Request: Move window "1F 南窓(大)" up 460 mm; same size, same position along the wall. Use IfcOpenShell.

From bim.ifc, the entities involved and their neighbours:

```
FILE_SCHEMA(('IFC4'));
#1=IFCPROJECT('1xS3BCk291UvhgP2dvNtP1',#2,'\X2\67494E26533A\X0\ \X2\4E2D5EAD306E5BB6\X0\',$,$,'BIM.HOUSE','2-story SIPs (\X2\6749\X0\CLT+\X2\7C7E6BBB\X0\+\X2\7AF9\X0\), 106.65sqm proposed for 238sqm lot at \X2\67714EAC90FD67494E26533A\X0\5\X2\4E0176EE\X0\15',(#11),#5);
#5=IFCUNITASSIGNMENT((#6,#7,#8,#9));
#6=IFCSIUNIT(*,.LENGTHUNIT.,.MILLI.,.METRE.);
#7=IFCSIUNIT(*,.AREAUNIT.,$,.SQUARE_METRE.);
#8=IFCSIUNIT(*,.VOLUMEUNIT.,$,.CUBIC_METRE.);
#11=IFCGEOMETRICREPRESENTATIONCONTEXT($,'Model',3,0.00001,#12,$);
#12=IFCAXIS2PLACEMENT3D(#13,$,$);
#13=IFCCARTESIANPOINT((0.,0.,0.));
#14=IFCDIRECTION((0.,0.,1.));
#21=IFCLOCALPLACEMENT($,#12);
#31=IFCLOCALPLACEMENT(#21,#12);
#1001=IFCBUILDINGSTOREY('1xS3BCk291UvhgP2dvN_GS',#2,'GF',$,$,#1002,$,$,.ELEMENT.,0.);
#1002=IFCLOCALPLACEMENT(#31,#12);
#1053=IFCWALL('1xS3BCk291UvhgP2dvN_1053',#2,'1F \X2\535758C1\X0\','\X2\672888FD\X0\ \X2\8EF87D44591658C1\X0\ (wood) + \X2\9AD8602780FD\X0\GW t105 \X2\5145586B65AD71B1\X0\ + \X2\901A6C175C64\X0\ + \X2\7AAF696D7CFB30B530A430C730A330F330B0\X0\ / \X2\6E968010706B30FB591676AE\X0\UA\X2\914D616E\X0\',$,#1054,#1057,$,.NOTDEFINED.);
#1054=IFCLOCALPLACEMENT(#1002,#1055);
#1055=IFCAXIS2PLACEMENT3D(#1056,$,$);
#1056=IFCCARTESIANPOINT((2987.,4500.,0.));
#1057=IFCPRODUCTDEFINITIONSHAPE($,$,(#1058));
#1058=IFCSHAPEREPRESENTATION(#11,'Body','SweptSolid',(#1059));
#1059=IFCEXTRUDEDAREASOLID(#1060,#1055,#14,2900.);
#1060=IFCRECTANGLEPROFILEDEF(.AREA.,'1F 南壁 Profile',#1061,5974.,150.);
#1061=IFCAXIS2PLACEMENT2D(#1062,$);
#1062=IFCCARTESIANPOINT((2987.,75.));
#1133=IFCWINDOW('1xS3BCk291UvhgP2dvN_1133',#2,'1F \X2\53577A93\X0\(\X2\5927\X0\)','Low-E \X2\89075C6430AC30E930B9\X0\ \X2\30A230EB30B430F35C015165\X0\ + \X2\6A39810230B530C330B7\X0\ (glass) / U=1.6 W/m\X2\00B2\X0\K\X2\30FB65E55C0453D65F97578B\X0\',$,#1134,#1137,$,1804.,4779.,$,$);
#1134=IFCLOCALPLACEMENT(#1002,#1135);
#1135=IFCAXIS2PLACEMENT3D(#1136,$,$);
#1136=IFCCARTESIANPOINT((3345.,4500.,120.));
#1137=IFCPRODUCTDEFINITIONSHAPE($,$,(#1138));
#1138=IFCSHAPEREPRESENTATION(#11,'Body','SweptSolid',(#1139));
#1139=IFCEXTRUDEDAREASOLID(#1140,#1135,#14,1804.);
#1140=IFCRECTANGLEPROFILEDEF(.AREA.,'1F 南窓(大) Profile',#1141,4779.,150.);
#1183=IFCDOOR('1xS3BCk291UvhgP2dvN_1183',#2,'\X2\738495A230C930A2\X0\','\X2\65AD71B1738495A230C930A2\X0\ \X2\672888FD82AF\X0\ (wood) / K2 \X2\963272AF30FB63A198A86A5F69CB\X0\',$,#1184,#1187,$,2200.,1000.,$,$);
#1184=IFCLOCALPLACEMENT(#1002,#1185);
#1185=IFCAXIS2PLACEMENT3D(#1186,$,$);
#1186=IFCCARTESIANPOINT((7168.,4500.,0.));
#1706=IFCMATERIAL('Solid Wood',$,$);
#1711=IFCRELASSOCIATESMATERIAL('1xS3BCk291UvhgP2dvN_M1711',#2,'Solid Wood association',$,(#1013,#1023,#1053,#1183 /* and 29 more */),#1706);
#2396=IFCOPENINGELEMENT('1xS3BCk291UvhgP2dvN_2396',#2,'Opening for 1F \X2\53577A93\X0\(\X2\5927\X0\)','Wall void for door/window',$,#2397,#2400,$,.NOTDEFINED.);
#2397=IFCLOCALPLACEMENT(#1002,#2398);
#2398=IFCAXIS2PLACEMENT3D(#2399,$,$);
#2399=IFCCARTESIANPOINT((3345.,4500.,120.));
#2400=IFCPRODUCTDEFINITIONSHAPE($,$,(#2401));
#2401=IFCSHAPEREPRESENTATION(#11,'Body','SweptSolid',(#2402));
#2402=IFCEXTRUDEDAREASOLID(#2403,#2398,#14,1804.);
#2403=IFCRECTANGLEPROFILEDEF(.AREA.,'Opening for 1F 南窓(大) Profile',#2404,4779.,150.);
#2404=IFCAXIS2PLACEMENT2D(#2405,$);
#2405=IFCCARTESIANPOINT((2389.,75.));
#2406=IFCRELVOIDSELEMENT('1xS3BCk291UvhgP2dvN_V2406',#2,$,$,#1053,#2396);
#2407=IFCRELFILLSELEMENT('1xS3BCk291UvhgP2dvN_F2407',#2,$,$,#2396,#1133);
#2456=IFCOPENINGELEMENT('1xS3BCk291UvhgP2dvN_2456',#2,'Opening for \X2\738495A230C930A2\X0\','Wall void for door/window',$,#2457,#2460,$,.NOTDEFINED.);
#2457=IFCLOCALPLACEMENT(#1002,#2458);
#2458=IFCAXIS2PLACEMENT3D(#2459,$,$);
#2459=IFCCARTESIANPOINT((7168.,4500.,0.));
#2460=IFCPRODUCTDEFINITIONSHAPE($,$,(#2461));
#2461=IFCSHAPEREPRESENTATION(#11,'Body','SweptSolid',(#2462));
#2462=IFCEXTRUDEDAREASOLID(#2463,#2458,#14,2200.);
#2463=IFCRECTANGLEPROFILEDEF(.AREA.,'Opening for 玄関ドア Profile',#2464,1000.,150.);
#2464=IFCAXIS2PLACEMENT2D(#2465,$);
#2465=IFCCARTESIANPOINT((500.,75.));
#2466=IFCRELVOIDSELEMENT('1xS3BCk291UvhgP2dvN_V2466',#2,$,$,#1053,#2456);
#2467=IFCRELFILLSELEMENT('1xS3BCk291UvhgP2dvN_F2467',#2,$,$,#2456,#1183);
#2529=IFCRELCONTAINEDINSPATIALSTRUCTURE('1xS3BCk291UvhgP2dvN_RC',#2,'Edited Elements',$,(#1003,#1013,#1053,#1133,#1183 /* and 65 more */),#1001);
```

```python
import numpy as np
import ifcopenshell
import ifcopenshell.api.geometry
import ifcopenshell.util.placement
import ifcopenshell.util.unit

model = ifcopenshell.open("bim.ifc")
unit_scale = ifcopenshell.util.unit.calculate_unit_scale(model)

window = model.by_guid("1xS3BCk291UvhgP2dvN_1133")
opening = window.FillsVoids[0].RelatingOpeningElement
dz = 460.0

shift = np.array([0.0, 0.0, dz])
# The window is not placed relative to its opening, so move both.
for product in (opening, window):
    matrix = ifcopenshell.util.placement.get_local_placement(product.ObjectPlacement)
    matrix[:3, 3] += shift
    ifcopenshell.api.geometry.edit_object_placement(model, product=product, matrix=matrix, is_si=False)

print(f"moved by {dz * unit_scale:+.3f} m")

model.write("bim-out.ifc")
```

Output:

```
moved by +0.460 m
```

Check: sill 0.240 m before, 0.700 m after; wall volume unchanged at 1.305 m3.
